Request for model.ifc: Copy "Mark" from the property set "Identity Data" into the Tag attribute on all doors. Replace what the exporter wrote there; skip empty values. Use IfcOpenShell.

First a look at what the model holds.

```python
import ifcopenshell
import ifcopenshell.util.element

model = ifcopenshell.open("model.ifc")
print(model.schema)
doors = model.by_type("IfcDoor")
print(len(doors), "doors")
for e in doors[:8]:
    source = ifcopenshell.util.element.get_pset(e, "Identity Data", "Mark")
    target = e.Tag
    print(e.id(), repr(source), repr(target), sep=" | ")
```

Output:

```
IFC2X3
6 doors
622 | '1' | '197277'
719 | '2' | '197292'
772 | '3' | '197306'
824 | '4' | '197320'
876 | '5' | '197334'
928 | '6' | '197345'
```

```python
import ifcopenshell
import ifcopenshell.util.element

model = ifcopenshell.open("model.ifc")

count = 0
for e in model.by_type("IfcDoor"):
    value = ifcopenshell.util.element.get_pset(e, "Identity Data", "Mark")
    current = e.Tag
    if not value or not value.strip() or current == value:
        continue
    e.Tag = value
    count += 1

print(count, "doors updated")

model.write("model_updated.ifc")
```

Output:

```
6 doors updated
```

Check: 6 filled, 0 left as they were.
